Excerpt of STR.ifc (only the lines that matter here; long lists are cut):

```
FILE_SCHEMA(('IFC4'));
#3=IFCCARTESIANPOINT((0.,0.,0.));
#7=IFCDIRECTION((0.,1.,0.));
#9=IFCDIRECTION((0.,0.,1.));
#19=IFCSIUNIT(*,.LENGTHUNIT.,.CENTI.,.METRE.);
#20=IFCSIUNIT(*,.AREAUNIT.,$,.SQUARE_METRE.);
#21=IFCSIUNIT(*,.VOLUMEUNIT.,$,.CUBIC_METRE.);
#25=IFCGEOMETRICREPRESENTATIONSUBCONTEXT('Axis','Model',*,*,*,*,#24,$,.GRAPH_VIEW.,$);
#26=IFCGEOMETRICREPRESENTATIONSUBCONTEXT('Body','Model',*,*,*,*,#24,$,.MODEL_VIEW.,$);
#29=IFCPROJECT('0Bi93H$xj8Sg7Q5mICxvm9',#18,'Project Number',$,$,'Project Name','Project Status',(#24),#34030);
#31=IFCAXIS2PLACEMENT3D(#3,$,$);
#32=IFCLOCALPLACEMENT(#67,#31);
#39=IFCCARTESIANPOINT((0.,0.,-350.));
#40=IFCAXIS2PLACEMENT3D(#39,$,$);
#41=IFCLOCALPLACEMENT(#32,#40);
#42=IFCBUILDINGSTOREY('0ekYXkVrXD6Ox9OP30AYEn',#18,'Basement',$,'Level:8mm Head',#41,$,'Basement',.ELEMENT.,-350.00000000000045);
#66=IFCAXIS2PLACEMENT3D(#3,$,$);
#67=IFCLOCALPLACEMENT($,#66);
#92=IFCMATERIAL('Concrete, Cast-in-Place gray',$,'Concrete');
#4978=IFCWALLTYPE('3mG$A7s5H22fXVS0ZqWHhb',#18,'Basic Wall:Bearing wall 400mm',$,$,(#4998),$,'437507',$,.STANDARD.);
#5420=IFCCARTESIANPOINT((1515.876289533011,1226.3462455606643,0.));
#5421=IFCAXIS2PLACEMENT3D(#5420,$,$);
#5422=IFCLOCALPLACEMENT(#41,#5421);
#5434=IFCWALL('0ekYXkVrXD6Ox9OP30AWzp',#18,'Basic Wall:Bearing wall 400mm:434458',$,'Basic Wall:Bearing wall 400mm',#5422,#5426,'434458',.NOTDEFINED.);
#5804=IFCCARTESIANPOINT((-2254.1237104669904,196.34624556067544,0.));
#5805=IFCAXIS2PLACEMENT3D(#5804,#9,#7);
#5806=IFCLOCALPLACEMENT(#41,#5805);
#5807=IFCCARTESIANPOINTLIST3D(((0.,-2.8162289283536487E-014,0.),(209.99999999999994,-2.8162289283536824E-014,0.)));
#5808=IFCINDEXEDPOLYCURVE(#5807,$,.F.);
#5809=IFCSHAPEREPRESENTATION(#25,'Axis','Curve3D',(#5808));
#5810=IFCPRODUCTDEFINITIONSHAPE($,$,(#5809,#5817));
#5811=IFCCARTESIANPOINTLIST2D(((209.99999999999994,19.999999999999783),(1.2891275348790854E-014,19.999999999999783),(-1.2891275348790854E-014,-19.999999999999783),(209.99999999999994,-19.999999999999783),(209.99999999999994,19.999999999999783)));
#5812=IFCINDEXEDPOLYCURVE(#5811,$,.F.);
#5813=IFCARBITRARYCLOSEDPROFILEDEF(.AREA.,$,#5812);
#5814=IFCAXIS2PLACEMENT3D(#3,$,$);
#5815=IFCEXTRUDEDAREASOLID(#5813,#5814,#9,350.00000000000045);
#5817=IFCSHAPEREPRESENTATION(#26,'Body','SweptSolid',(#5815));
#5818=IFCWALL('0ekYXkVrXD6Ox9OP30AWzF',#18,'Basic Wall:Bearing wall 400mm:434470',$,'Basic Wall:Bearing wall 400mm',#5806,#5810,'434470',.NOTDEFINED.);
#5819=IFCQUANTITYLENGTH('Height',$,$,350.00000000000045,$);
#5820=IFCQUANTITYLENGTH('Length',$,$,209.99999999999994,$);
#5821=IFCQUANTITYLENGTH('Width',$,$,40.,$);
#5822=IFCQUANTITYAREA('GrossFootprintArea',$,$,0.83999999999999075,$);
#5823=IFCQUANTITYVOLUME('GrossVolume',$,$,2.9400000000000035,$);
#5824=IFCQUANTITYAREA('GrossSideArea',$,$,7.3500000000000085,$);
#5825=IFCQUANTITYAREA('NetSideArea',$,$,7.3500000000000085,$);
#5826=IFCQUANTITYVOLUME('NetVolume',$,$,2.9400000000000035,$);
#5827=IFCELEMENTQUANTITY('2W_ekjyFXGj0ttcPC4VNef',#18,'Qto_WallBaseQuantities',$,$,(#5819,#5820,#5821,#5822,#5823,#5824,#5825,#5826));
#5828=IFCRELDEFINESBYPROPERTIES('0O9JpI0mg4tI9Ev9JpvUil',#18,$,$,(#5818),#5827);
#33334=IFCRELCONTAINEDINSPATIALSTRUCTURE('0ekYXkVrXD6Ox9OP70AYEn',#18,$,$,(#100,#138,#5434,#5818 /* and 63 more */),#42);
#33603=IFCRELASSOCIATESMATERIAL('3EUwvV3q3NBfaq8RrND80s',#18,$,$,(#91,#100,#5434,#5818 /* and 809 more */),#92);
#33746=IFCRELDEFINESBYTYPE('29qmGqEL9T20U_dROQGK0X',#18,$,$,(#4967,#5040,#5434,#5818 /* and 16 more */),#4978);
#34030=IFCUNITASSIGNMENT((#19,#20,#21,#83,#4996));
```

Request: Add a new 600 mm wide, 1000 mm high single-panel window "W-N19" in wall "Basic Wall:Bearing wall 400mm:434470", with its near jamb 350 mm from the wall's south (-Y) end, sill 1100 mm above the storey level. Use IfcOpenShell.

```python
import numpy as np
import ifcopenshell
import ifcopenshell.api.feature
import ifcopenshell.api.geometry
import ifcopenshell.api.pset
import ifcopenshell.api.root
import ifcopenshell.api.spatial
import ifcopenshell.geom
import ifcopenshell.util.element
import ifcopenshell.util.placement
import ifcopenshell.util.representation
import ifcopenshell.util.shape
import ifcopenshell.util.unit

model = ifcopenshell.open("STR.ifc")
unit_scale = ifcopenshell.util.unit.calculate_unit_scale(model)
area_scale = ifcopenshell.util.unit.calculate_unit_scale(model, "AREAUNIT")
volume_scale = ifcopenshell.util.unit.calculate_unit_scale(model, "VOLUMEUNIT")
settings = ifcopenshell.geom.settings()


def volume(element):
    """Net volume in cubic metres, openings subtracted."""
    shape = ifcopenshell.geom.create_shape(settings, element)
    return ifcopenshell.util.shape.get_volume(shape.geometry)


wall = model.by_guid("0ekYXkVrXD6Ox9OP30AWzF")
storey = ifcopenshell.util.element.get_container(wall, ifc_class="IfcBuildingStorey")
context = ifcopenshell.util.representation.get_context(model, "Model", "Body", "MODEL_VIEW")
before = volume(wall)

width, height, from_end, sill = 0.6, 1, 0.35, 1.1  # metres

# The wall runs along its own X axis, and the end named is its -X end.
wall_shape = ifcopenshell.geom.create_shape(settings, wall)
x, y, z = ifcopenshell.util.shape.get_vertices(wall_shape.geometry).T
start = x.min() + from_end
face, thickness = float(y.min()), float(y.max() - y.min())
wall_matrix = ifcopenshell.util.placement.get_local_placement(wall.ObjectPlacement)
level = ifcopenshell.util.placement.get_local_placement(storey.ObjectPlacement)[2, 3]


def in_wall(x, y):
    """Placement at x, y metres in the wall's axes, at sill height."""
    matrix = wall_matrix.copy()
    matrix[:, 3] = wall_matrix @ np.array([x / unit_scale, y / unit_scale, 0.0, 1.0])
    matrix[2, 3] = level + sill / unit_scale
    return matrix


# Opening: a box that overshoots both wall faces by 50 mm.
opening = ifcopenshell.api.root.create_entity(model, ifc_class="IfcOpeningElement", predefined_type="OPENING")
box = ifcopenshell.api.geometry.add_wall_representation(
    model, context=context, length=width, height=height, thickness=thickness + 0.1
)
ifcopenshell.api.geometry.assign_representation(model, product=opening, representation=box)
ifcopenshell.api.geometry.edit_object_placement(model, product=opening, matrix=in_wall(start, face - 0.05), is_si=False)
ifcopenshell.api.feature.add_feature(model, feature=opening, element=wall)

window = ifcopenshell.api.root.create_entity(model, ifc_class="IfcWindow", name="W-N19", predefined_type="WINDOW")
window.OverallWidth, window.OverallHeight = width / unit_scale, height / unit_scale
window.PartitioningType = "SINGLE_PANEL"
body = ifcopenshell.api.geometry.add_window_representation(
    model,
    context=context,
    overall_width=window.OverallWidth,
    overall_height=window.OverallHeight,
    partition_type="SINGLE_PANEL",
)
ifcopenshell.api.geometry.assign_representation(model, product=window, representation=body)
ifcopenshell.api.spatial.assign_container(model, products=[window], relating_structure=storey)
ifcopenshell.api.feature.add_filling(model, opening=opening, element=window)

# Centre the window in the wall's thickness.
ifcopenshell.api.geometry.edit_object_placement(model, product=window, matrix=in_wall(start, face), is_si=False)
window_shape = ifcopenshell.geom.create_shape(settings, window)
depth = ifcopenshell.util.shape.get_vertices(window_shape.geometry)[:, 1]
offset = face + thickness / 2 - (depth.min() + depth.max()) / 2
ifcopenshell.api.geometry.edit_object_placement(model, product=window, matrix=in_wall(start, offset), is_si=False)

after = volume(wall)

# Update the wall's stored quantities.
qto = model.by_id(ifcopenshell.util.element.get_pset(wall, "Qto_WallBaseQuantities", should_inherit=False)["id"])
ifcopenshell.api.pset.edit_qto(model, qto=qto, properties={
    "NetSideArea": after / thickness / area_scale,
    "NetVolume": after / volume_scale,
})

print(f"wall volume {before:.3f} -> {after:.3f} m3")

model.write("STR_rev.ifc")
```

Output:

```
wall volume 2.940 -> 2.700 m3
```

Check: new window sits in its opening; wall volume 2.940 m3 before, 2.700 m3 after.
